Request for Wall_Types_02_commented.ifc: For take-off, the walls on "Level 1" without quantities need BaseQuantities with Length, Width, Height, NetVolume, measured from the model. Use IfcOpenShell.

First a look at what the model holds.

```python
import ifcopenshell
import ifcopenshell.util.element
import ifcopenshell.util.unit

model = ifcopenshell.open("Wall_Types_02_commented.ifc")
print(model.schema)
for unit_type in ("LENGTHUNIT", "AREAUNIT", "VOLUMEUNIT"):
    print(unit_type, ifcopenshell.util.unit.calculate_unit_scale(model, unit_type))
storey = next(s for s in model.by_type("IfcBuildingStorey") if s.Name == "Level 1")
walls = [e for e in ifcopenshell.util.element.get_decomposition(storey) if e.is_a("IfcWall")]
for e in sorted(walls, key=lambda e: e.id()):
    print(e.id(), e.is_a(), e.Name, list(ifcopenshell.util.element.get_psets(e, qtos_only=True)), sep=" | ")
```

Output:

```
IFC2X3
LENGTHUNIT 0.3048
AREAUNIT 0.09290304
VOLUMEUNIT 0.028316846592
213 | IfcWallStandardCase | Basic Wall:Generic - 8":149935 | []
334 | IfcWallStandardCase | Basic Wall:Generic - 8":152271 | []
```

```python
import ifcopenshell
import ifcopenshell.api.pset
import ifcopenshell.geom
import ifcopenshell.util.element
import ifcopenshell.util.shape
import ifcopenshell.util.unit

model = ifcopenshell.open("Wall_Types_02_commented.ifc")
unit_scale = ifcopenshell.util.unit.calculate_unit_scale(model)
volume_scale = ifcopenshell.util.unit.calculate_unit_scale(model, "VOLUMEUNIT")
settings = ifcopenshell.geom.settings()

storey = next(s for s in model.by_type("IfcBuildingStorey") if s.Name == "Level 1")
walls = [e for e in ifcopenshell.util.element.get_decomposition(storey) if e.is_a("IfcWall")]

for e in sorted(walls, key=lambda e: e.id()):
    if ifcopenshell.util.element.get_psets(e, qtos_only=True, should_inherit=False):
        continue
    # Geometry comes back in metres, in the element's own axes.
    shape = ifcopenshell.geom.create_shape(settings, e)
    values = {
        "Length": ifcopenshell.util.shape.get_x(shape.geometry) / unit_scale,
        "Width": ifcopenshell.util.shape.get_y(shape.geometry) / unit_scale,
        "Height": ifcopenshell.util.shape.get_z(shape.geometry) / unit_scale,
        "NetVolume": ifcopenshell.util.shape.get_volume(shape.geometry) / volume_scale,
    }
    qto = ifcopenshell.api.pset.add_qto(model, product=e, name="BaseQuantities")
    ifcopenshell.api.pset.edit_qto(model, qto=qto, properties=values)
    print(e.id(), {k: round(v, 3) for k, v in values.items()})

model.write("Wall_Types_02_commented_rev.ifc")
```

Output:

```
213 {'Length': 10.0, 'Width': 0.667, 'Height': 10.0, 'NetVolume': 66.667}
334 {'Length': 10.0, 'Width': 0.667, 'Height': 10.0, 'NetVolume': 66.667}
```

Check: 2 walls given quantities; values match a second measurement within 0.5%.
